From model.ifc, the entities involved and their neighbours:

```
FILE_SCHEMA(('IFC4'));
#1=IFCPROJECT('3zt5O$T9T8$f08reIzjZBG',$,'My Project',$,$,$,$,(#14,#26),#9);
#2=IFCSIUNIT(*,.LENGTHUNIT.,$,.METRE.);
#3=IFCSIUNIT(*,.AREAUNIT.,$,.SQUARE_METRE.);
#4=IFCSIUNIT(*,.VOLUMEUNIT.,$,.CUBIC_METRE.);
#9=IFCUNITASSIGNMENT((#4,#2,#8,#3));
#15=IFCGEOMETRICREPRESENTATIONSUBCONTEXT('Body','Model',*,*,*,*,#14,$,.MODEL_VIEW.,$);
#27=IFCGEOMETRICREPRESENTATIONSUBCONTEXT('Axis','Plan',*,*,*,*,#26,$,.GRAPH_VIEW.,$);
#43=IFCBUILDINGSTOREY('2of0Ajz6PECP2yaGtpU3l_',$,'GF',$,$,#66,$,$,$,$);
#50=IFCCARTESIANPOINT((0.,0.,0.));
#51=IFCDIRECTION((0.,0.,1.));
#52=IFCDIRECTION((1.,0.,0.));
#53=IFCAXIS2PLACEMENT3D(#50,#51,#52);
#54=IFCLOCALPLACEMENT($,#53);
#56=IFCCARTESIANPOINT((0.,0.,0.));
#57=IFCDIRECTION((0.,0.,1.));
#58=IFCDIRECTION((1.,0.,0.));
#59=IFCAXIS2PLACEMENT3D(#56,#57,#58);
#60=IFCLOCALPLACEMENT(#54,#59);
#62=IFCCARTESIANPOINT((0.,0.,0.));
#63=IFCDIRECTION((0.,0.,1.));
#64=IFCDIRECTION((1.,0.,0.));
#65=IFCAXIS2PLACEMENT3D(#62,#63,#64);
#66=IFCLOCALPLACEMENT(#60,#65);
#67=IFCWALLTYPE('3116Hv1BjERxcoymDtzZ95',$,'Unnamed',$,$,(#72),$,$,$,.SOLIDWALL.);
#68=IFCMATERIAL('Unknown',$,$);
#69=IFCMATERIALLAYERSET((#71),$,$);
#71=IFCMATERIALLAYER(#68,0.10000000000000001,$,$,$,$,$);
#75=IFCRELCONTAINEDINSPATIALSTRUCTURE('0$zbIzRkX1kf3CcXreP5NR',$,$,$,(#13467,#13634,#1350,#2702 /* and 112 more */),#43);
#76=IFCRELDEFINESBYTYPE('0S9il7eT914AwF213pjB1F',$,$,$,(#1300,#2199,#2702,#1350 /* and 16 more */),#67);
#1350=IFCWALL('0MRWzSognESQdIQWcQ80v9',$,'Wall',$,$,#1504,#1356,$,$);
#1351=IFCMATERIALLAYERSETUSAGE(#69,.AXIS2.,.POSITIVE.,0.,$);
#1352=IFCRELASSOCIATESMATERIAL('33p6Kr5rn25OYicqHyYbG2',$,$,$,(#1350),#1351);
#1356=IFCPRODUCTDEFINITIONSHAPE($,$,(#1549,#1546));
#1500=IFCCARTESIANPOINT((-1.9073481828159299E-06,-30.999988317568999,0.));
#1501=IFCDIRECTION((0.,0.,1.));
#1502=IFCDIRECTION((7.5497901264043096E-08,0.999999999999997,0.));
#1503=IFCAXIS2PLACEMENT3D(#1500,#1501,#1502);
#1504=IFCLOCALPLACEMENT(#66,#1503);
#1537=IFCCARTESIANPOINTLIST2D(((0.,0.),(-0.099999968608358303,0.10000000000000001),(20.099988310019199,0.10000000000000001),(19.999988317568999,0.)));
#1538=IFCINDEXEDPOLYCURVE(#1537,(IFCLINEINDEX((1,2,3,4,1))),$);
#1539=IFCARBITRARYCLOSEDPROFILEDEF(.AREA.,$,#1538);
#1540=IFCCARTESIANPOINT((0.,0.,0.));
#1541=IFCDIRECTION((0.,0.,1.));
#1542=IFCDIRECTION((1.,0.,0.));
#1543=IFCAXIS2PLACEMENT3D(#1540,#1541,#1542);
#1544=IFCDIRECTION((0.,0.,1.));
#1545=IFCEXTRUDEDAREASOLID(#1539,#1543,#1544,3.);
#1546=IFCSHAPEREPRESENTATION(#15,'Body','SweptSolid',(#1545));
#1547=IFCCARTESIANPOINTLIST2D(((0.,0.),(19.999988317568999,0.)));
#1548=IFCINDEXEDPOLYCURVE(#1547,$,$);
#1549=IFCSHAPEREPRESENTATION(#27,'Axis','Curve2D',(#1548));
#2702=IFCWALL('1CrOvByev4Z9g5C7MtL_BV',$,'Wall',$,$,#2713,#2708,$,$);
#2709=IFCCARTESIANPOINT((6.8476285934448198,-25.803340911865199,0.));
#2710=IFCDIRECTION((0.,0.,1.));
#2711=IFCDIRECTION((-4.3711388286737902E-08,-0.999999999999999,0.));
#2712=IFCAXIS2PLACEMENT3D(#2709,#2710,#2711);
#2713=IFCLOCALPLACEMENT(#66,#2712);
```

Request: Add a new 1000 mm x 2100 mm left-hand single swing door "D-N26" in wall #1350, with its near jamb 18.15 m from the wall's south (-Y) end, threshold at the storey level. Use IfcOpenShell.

```python
import numpy as np
import ifcopenshell
import ifcopenshell.api.feature
import ifcopenshell.api.geometry
import ifcopenshell.api.root
import ifcopenshell.api.spatial
import ifcopenshell.geom
import ifcopenshell.util.element
import ifcopenshell.util.placement
import ifcopenshell.util.representation
import ifcopenshell.util.shape
import ifcopenshell.util.unit

model = ifcopenshell.open("model.ifc")
unit_scale = ifcopenshell.util.unit.calculate_unit_scale(model)
settings = ifcopenshell.geom.settings()


def volume(element):
    """Net volume in cubic metres, openings subtracted."""
    shape = ifcopenshell.geom.create_shape(settings, element)
    return ifcopenshell.util.shape.get_volume(shape.geometry)


wall = model.by_guid("0MRWzSognESQdIQWcQ80v9")
storey = ifcopenshell.util.element.get_container(wall, ifc_class="IfcBuildingStorey")
context = ifcopenshell.util.representation.get_context(model, "Model", "Body", "MODEL_VIEW")
before = volume(wall)

width, height, from_end, sill = 1, 2.1, 18.15, 0.0  # metres

# The wall runs along its own X axis, and the end named is its -X end.
wall_shape = ifcopenshell.geom.create_shape(settings, wall)
x, y, z = ifcopenshell.util.shape.get_vertices(wall_shape.geometry).T
start = x.min() + from_end
face, thickness = float(y.min()), float(y.max() - y.min())
wall_matrix = ifcopenshell.util.placement.get_local_placement(wall.ObjectPlacement)
level = ifcopenshell.util.placement.get_local_placement(storey.ObjectPlacement)[2, 3]


def in_wall(x, y):
    """Placement at x, y metres in the wall's axes, at sill height."""
    matrix = wall_matrix.copy()
    matrix[:, 3] = wall_matrix @ np.array([x / unit_scale, y / unit_scale, 0.0, 1.0])
    matrix[2, 3] = level + sill / unit_scale
    return matrix


# Opening: a box that overshoots both wall faces by 50 mm.
opening = ifcopenshell.api.root.create_entity(model, ifc_class="IfcOpeningElement", predefined_type="OPENING")
box = ifcopenshell.api.geometry.add_wall_representation(
    model, context=context, length=width, height=height, thickness=thickness + 0.1
)
ifcopenshell.api.geometry.assign_representation(model, product=opening, representation=box)
ifcopenshell.api.geometry.edit_object_placement(model, product=opening, matrix=in_wall(start, face - 0.05), is_si=False)
ifcopenshell.api.feature.add_feature(model, feature=opening, element=wall)

door = ifcopenshell.api.root.create_entity(model, ifc_class="IfcDoor", name="D-N26", predefined_type="DOOR")
door.OverallWidth, door.OverallHeight = width / unit_scale, height / unit_scale
door.OperationType = "SINGLE_SWING_LEFT"
body = ifcopenshell.api.geometry.add_door_representation(
    model,
    context=context,
    overall_width=door.OverallWidth,
    overall_height=door.OverallHeight,
    operation_type="SINGLE_SWING_LEFT",
    lining_properties={"LiningDepth": thickness / unit_scale, "ThresholdDepth": thickness / unit_scale},
)
ifcopenshell.api.geometry.assign_representation(model, product=door, representation=body)
ifcopenshell.api.spatial.assign_container(model, products=[door], relating_structure=storey)
ifcopenshell.api.feature.add_filling(model, opening=opening, element=door)

# The lining spans the wall, so the door starts at the wall face.
ifcopenshell.api.geometry.edit_object_placement(model, product=door, matrix=in_wall(start, face), is_si=False)

after = volume(wall)

print(f"wall volume {before:.3f} -> {after:.3f} m3")

model.write("model_updated.ifc")
```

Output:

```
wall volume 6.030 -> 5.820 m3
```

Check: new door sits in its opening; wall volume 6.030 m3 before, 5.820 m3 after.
